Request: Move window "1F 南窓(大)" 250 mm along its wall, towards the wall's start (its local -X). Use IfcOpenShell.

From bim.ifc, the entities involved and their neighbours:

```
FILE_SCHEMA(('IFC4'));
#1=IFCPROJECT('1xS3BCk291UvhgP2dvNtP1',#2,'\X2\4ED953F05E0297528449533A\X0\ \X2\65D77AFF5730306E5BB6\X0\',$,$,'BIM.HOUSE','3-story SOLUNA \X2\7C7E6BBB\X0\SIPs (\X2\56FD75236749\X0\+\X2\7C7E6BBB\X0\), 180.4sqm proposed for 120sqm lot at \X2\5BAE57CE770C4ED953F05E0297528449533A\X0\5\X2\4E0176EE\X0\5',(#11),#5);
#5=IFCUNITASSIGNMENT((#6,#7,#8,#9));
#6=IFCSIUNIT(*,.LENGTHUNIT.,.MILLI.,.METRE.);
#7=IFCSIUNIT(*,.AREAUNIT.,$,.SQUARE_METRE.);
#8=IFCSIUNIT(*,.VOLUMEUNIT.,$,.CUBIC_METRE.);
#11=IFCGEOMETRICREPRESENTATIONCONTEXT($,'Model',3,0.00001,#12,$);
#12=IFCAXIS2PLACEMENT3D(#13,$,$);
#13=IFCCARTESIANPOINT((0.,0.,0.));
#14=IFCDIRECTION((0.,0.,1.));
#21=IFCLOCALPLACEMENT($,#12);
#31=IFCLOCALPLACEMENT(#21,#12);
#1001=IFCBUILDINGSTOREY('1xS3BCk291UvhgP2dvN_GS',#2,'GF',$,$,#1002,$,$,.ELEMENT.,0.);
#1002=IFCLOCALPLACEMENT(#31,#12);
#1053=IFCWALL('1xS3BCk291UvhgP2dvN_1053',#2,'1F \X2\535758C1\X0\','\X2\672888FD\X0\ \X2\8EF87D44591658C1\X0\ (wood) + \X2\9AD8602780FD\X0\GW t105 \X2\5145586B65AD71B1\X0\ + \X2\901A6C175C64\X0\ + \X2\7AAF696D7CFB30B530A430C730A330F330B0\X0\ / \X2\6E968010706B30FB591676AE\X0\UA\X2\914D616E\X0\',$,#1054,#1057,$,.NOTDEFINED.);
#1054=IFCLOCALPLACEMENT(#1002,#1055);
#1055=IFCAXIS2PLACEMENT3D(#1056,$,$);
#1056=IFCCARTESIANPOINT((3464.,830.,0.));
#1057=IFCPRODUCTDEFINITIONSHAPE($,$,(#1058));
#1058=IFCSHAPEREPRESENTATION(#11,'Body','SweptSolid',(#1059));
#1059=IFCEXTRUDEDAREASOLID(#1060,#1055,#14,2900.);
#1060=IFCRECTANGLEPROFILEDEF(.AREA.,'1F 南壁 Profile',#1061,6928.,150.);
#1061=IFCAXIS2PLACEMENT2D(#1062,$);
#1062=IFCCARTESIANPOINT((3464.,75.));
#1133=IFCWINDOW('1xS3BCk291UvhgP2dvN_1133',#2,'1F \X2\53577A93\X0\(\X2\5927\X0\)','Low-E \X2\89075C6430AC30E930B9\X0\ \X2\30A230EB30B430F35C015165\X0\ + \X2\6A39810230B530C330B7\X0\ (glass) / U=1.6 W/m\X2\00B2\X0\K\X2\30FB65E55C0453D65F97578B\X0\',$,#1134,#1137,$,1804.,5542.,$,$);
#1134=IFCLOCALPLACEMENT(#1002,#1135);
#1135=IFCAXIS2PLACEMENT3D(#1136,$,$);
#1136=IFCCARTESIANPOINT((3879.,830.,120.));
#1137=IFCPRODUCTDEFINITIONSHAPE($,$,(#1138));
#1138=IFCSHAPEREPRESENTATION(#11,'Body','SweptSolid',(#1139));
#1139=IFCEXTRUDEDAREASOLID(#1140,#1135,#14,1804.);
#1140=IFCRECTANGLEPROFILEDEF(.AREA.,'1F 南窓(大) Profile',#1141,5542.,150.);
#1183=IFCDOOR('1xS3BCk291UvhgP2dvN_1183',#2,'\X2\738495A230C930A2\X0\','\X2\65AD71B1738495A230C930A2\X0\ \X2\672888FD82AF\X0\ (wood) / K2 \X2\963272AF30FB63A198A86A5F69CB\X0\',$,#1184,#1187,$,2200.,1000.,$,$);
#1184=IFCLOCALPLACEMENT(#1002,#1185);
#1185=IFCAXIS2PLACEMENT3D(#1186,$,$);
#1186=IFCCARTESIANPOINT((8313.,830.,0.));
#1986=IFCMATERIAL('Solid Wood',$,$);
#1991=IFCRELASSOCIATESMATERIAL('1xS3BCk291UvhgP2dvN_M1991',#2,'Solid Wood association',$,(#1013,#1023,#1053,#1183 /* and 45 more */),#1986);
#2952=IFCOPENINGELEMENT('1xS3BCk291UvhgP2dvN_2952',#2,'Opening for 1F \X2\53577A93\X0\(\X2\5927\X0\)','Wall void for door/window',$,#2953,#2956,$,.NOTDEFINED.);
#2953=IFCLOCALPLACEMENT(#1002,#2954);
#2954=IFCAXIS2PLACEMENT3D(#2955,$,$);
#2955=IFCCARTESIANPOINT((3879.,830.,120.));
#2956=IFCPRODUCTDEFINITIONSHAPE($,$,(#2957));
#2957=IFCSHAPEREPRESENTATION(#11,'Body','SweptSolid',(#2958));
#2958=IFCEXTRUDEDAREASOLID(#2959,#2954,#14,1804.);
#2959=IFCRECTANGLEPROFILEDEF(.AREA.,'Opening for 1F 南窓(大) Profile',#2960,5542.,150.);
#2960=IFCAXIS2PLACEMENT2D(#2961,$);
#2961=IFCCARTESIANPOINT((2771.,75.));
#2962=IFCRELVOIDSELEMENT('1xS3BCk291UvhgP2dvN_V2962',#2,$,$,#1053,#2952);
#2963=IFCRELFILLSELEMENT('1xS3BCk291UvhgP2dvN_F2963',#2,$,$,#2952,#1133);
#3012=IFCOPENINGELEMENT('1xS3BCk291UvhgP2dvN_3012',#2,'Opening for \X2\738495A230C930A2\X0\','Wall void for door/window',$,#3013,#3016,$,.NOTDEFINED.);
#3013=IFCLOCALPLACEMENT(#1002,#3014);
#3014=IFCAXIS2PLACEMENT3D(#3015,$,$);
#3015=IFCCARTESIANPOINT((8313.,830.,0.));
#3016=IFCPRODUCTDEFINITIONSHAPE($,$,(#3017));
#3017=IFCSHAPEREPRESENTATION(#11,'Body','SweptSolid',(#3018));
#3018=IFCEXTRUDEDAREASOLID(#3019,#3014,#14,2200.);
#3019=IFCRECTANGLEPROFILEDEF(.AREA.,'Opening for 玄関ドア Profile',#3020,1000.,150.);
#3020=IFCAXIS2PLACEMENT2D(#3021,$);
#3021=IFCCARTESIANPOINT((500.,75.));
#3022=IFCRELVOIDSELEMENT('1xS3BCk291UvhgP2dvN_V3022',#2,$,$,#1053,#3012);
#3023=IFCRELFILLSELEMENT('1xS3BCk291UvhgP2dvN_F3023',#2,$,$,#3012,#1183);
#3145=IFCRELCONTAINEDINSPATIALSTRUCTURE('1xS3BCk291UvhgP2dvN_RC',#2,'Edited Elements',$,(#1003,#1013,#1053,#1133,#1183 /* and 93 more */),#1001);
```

```python
import ifcopenshell
import ifcopenshell.api.geometry
import ifcopenshell.util.placement

model = ifcopenshell.open("bim.ifc")

window = model.by_guid("1xS3BCk291UvhgP2dvN_1133")
opening = window.FillsVoids[0].RelatingOpeningElement
wall = opening.VoidsElements[0].RelatingBuildingElement

wall_matrix = ifcopenshell.util.placement.get_local_placement(wall.ObjectPlacement)
shift = wall_matrix[:3, 0] * -250.0
before = ifcopenshell.util.placement.get_local_placement(window.ObjectPlacement)[:3, 3].copy()

# The window is not placed relative to its opening, so move both.
for product in (opening, window):
    matrix = ifcopenshell.util.placement.get_local_placement(product.ObjectPlacement)
    matrix[:3, 3] += shift
    ifcopenshell.api.geometry.edit_object_placement(model, product=product, matrix=matrix, is_si=False)

after = ifcopenshell.util.placement.get_local_placement(window.ObjectPlacement)[:3, 3]
print("window moved by", (after - before).round(3) + 0.0)

model.write("bim_v2.ifc")
```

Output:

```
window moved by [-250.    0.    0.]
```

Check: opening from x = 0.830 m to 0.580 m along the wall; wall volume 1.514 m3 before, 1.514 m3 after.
